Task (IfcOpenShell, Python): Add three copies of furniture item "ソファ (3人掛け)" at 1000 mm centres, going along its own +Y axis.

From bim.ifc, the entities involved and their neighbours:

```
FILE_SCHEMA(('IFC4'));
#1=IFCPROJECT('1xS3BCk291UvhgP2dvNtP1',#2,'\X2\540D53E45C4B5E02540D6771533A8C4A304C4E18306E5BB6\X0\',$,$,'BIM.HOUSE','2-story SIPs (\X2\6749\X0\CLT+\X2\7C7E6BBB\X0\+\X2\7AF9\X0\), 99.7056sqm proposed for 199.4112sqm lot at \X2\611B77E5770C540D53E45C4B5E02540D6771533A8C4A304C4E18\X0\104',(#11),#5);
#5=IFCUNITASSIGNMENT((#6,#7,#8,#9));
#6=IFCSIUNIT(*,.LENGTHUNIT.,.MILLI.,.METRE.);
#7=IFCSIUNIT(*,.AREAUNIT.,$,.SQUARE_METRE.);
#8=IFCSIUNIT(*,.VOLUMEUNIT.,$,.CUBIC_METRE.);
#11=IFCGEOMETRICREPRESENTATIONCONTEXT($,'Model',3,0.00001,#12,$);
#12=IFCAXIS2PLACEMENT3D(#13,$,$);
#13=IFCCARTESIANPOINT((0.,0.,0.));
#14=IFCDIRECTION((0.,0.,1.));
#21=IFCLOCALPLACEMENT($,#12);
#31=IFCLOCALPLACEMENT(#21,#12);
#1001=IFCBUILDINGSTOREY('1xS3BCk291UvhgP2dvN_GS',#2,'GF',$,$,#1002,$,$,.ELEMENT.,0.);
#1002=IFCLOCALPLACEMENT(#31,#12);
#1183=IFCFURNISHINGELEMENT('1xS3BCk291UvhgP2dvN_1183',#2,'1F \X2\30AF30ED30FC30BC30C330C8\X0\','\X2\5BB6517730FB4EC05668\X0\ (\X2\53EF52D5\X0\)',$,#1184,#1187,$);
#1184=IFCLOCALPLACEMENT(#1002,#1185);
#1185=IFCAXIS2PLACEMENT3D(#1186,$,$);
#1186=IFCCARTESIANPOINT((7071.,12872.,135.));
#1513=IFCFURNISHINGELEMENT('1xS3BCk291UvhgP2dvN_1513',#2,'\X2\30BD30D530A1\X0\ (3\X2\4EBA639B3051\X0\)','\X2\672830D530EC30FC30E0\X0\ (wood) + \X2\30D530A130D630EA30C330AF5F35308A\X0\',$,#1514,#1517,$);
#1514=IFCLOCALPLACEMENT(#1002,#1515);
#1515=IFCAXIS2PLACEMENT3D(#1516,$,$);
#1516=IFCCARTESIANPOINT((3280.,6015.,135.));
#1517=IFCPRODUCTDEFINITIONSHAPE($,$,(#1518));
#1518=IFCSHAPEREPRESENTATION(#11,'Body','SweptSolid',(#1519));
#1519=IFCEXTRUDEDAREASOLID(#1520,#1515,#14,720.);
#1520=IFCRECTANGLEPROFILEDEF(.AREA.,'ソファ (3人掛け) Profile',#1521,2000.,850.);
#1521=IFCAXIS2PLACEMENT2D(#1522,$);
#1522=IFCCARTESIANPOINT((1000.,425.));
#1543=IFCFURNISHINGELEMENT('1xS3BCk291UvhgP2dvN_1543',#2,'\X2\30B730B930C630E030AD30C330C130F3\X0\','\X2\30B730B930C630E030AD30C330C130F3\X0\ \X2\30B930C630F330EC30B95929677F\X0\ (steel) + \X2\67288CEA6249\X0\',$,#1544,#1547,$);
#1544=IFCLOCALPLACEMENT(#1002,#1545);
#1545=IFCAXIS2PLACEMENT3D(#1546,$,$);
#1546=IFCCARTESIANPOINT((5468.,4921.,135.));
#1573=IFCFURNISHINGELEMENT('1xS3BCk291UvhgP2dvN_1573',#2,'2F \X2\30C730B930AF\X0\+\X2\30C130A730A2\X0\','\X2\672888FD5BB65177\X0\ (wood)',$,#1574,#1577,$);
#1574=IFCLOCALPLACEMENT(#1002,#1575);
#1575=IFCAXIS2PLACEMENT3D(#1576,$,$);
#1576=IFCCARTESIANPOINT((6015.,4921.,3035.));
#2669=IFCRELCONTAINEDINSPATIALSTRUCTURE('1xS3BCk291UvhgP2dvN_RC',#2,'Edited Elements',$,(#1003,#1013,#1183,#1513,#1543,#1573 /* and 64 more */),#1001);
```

```python
import ifcopenshell
import ifcopenshell.api.geometry
import ifcopenshell.api.root
import ifcopenshell.util.element
import ifcopenshell.util.placement

model = ifcopenshell.open("bim.ifc")


def reuse_history(source, copy):
    """copy_class also copies each property set's owner history, people and application; keep the originals."""
    for rel in copy.IsDefinedBy:
        if rel.is_a("IfcRelDefinesByProperties") and (history := rel.RelatingPropertyDefinition.OwnerHistory):
            rel.RelatingPropertyDefinition.OwnerHistory = source.OwnerHistory
            ifcopenshell.util.element.remove_deep2(model, history)


source = model.by_guid("1xS3BCk291UvhgP2dvN_1513")
base = ifcopenshell.util.placement.get_local_placement(source.ObjectPlacement)
step = base[:3, 1] * 1000.0

for i in range(1, 4):
    copy = ifcopenshell.api.root.copy_class(model, product=source)
    copy.Representation = ifcopenshell.util.element.copy_deep(
        model, source.Representation, exclude=["IfcGeometricRepresentationContext", "IfcRepresentationMap"]
    )
    reuse_history(source, copy)
    matrix = base.copy()
    matrix[:3, 3] += i * step
    print("added at", matrix[:3, 3].round(3) + 0.0)
    ifcopenshell.api.geometry.edit_object_placement(model, product=copy, matrix=matrix, is_si=False)

model.write("bim-out.ifc")
```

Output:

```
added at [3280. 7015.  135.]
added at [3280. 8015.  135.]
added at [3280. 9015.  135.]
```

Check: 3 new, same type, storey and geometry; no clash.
